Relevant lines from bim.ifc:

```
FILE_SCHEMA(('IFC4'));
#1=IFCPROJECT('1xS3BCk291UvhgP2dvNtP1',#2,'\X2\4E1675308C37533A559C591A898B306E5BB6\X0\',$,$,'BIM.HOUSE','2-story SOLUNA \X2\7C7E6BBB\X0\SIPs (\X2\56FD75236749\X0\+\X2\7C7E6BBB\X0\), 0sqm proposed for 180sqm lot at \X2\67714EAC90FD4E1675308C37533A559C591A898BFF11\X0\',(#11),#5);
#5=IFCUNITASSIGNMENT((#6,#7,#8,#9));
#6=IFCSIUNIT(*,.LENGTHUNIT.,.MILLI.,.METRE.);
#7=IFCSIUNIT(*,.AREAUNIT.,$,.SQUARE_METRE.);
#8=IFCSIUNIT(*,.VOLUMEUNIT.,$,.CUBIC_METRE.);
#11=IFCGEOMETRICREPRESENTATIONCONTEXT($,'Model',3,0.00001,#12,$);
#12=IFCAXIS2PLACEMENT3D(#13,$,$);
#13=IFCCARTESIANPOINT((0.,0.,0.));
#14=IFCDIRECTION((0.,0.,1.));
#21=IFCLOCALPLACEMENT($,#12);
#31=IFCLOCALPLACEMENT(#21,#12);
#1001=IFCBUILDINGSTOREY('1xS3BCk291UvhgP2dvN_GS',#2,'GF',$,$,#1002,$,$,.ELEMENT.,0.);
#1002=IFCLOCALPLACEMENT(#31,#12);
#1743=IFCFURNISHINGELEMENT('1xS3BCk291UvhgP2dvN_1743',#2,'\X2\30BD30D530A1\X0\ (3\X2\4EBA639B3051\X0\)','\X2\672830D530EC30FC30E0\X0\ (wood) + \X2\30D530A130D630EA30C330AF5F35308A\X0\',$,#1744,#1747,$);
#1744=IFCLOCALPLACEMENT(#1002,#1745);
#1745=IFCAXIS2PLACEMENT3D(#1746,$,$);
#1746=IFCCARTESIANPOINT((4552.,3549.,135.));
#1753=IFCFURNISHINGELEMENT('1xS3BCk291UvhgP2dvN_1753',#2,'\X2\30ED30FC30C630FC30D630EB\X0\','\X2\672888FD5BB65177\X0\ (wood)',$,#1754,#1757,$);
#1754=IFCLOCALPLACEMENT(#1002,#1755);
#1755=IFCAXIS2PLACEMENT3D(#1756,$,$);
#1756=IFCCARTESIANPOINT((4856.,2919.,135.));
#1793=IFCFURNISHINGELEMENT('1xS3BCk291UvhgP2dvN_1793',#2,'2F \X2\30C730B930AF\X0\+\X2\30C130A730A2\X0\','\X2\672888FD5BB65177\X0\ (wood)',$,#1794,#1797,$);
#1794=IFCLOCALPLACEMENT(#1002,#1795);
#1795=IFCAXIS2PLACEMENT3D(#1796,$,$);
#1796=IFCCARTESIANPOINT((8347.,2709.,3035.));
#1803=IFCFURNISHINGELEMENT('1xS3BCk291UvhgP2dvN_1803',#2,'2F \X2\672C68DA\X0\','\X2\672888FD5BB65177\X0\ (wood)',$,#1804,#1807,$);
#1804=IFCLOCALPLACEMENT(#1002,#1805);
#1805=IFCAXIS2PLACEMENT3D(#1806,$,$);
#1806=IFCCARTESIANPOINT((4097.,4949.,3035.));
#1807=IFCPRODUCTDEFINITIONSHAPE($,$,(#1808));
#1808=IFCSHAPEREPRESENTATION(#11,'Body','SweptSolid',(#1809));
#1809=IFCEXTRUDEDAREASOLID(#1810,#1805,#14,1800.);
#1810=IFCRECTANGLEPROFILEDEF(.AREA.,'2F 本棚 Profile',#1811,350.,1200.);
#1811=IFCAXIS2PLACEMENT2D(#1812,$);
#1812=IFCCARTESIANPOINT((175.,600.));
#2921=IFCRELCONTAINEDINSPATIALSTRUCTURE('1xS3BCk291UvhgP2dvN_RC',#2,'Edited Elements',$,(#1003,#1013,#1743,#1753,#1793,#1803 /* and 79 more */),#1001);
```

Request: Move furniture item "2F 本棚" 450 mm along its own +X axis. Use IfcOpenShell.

```python
import ifcopenshell
import ifcopenshell.api.geometry
import ifcopenshell.util.placement
import ifcopenshell.util.unit

model = ifcopenshell.open("bim.ifc")
unit_scale = ifcopenshell.util.unit.calculate_unit_scale(model)

item = model.by_guid("1xS3BCk291UvhgP2dvN_1803")
matrix = ifcopenshell.util.placement.get_local_placement(item.ObjectPlacement)
matrix[:3, 3] += matrix[:3, 0] * 0.45 / unit_scale
ifcopenshell.api.geometry.edit_object_placement(model, product=item, matrix=matrix, is_si=False)

print(ifcopenshell.util.placement.get_local_placement(item.ObjectPlacement).round(3) + 0.0)

model.write("bim_v2.ifc")
```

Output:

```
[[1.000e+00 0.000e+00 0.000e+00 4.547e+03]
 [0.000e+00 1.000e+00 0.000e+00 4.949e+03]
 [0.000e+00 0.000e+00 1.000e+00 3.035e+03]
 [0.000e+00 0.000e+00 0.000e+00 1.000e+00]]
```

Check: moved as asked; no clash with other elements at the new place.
